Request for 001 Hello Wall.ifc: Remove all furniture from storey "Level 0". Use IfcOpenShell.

First a look at what the model holds.

```python
import ifcopenshell
import ifcopenshell.util.element

model = ifcopenshell.open("001 Hello Wall.ifc")
print(model.schema)
storey = next(s for s in model.by_type("IfcBuildingStorey") if s.Name == "Level 0")
furniture = [e for e in ifcopenshell.util.element.get_decomposition(storey) if e.is_a("IfcFurnishingElement")]
seen = {}
for e in furniture:
    element_type = ifcopenshell.util.element.get_type(e)
    name = element_type.Name if element_type not in (None, e) else None
    seen[name] = seen.get(name, 0) + 1
for name, count in sorted(seen.items(), key=str):
    print(count, "x", name)
```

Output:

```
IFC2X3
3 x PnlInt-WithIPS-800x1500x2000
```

```python
import ifcopenshell
import ifcopenshell.api.root
import ifcopenshell.util.element

model = ifcopenshell.open("001 Hello Wall.ifc")

storey = next(s for s in model.by_type("IfcBuildingStorey") if s.Name == "Level 0")
furniture = [e for e in ifcopenshell.util.element.get_decomposition(storey) if e.is_a("IfcFurnishingElement")]

for e in furniture:
    ifcopenshell.api.root.remove_product(model, product=e)
print(len(furniture), "removed")

model.write("001 Hello Wall_edited.ifc")
```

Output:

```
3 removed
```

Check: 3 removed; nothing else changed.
